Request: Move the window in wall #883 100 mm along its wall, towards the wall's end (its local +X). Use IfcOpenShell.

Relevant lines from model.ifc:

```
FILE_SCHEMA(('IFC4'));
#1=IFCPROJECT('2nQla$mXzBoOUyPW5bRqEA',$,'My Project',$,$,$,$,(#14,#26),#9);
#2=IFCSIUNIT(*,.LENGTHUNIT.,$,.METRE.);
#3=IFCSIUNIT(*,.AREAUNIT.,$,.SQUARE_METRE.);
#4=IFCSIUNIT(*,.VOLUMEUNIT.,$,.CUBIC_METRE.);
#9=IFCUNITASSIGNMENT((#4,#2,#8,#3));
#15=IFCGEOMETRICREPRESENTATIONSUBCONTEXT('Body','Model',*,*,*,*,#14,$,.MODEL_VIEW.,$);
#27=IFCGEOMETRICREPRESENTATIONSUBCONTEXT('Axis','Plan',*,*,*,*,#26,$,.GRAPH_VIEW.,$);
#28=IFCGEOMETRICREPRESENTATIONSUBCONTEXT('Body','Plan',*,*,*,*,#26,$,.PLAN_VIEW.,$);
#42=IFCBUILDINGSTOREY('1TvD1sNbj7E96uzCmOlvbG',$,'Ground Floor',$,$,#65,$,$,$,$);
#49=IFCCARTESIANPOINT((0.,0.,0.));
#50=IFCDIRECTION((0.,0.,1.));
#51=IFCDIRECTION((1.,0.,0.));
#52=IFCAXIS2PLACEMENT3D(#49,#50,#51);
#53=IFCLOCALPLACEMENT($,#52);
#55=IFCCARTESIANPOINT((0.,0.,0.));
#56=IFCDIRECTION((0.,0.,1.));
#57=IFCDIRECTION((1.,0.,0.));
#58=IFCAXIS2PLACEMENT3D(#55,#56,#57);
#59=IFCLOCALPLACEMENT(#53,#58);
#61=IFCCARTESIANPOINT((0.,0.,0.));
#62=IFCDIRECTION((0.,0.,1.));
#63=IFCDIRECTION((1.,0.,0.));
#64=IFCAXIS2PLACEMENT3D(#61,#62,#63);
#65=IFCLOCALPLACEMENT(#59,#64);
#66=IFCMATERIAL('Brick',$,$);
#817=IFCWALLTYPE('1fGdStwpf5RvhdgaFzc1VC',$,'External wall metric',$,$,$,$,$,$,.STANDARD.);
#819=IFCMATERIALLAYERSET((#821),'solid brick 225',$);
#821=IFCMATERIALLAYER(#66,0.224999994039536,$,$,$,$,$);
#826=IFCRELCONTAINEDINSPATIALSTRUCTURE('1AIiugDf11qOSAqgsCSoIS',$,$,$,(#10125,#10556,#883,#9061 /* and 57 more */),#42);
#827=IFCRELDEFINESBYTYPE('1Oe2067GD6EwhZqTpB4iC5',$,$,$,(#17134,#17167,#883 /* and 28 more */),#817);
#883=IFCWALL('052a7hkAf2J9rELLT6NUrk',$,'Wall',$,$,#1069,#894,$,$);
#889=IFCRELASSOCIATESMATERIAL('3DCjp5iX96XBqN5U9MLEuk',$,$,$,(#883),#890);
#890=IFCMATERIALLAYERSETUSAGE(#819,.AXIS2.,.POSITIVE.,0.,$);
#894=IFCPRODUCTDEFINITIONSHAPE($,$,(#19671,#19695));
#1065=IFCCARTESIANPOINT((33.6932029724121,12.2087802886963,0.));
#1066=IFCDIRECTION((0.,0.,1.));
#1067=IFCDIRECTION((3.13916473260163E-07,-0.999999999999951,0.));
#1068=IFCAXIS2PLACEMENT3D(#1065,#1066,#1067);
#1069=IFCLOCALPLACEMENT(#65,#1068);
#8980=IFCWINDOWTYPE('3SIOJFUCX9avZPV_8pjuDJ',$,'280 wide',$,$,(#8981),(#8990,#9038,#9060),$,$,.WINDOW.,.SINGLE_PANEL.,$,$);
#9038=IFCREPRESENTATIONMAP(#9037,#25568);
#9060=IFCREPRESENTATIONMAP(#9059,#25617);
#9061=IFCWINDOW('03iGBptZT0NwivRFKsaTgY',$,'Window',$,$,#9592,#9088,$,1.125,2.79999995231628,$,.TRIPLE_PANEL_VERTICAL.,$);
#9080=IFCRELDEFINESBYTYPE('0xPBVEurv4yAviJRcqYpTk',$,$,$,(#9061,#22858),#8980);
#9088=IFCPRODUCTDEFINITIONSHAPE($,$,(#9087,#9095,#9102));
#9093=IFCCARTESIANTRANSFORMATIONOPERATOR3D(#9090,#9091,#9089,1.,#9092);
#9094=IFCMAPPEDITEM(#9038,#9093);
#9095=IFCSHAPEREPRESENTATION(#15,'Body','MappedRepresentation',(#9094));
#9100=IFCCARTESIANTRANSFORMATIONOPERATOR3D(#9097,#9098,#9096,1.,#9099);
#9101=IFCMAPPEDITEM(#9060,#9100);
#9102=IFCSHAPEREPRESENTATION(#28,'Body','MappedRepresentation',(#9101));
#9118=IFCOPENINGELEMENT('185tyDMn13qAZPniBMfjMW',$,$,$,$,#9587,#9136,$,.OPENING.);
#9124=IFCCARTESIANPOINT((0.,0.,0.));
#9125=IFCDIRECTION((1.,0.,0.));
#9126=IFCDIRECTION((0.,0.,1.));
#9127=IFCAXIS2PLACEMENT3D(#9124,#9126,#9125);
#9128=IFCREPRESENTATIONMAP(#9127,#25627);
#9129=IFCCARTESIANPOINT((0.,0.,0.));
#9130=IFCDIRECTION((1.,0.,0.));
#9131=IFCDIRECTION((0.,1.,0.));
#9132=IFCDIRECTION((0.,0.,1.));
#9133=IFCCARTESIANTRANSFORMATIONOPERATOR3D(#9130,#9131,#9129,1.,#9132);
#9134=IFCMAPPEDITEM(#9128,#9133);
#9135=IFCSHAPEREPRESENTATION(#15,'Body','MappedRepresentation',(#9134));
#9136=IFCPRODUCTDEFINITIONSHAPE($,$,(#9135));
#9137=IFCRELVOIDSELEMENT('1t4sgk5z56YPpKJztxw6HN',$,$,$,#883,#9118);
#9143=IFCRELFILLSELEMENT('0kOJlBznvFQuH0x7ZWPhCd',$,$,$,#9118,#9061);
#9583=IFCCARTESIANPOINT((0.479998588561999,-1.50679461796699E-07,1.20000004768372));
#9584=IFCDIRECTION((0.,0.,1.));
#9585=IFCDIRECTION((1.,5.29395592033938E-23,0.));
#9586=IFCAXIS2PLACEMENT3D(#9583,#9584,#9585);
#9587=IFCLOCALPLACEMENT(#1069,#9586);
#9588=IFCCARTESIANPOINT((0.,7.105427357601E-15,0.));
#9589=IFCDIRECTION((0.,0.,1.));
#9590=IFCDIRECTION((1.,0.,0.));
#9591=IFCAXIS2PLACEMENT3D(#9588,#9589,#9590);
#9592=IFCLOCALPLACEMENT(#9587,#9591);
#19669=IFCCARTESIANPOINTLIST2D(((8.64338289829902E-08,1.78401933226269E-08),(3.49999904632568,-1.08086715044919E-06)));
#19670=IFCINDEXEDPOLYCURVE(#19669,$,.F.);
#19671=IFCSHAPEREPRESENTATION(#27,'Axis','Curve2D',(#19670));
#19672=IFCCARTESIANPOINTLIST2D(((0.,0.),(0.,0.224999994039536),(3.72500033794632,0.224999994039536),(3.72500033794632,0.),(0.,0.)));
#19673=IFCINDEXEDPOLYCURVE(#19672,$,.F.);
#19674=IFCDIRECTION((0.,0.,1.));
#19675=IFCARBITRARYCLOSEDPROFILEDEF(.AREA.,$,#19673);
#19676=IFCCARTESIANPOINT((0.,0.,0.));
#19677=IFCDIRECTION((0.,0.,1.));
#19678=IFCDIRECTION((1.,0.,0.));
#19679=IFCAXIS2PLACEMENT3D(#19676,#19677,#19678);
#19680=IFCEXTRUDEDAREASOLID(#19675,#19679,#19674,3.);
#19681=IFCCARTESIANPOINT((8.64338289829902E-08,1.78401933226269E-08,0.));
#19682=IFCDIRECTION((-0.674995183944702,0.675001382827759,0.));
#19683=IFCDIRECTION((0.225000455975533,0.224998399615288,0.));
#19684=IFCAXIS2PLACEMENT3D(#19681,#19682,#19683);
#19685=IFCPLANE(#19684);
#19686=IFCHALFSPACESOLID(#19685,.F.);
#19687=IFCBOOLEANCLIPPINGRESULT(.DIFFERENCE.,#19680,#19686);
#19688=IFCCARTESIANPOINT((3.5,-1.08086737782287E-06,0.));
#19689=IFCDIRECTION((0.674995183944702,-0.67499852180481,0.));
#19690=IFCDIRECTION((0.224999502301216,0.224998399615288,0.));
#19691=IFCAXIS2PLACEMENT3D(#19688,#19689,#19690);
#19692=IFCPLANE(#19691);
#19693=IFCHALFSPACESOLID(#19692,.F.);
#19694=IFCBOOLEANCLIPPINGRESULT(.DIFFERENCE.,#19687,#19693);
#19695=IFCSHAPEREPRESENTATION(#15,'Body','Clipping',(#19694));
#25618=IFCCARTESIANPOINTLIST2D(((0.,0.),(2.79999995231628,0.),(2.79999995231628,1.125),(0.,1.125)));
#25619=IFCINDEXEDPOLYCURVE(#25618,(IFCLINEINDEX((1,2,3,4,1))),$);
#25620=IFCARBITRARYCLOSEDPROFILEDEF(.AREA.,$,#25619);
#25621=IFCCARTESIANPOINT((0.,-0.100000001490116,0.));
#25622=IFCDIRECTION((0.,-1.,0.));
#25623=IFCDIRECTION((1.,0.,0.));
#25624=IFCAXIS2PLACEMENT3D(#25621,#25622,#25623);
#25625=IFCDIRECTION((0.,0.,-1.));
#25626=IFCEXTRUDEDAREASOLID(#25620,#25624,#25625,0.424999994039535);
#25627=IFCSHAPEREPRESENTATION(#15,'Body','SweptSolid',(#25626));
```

```python
import ifcopenshell
import ifcopenshell.api.geometry
import ifcopenshell.util.placement
import ifcopenshell.util.unit

model = ifcopenshell.open("model.ifc")
unit_scale = ifcopenshell.util.unit.calculate_unit_scale(model)

window = model.by_guid("03iGBptZT0NwivRFKsaTgY")
opening = window.FillsVoids[0].RelatingOpeningElement
wall = opening.VoidsElements[0].RelatingBuildingElement

wall_matrix = ifcopenshell.util.placement.get_local_placement(wall.ObjectPlacement)
shift = wall_matrix[:3, 0] * 0.1 / unit_scale
before = ifcopenshell.util.placement.get_local_placement(window.ObjectPlacement)[:3, 3].copy()

# The window is placed relative to its opening, so it follows when the opening moves.
matrix = ifcopenshell.util.placement.get_local_placement(opening.ObjectPlacement)
matrix[:3, 3] += shift
ifcopenshell.api.geometry.edit_object_placement(
    model, product=opening, matrix=matrix, is_si=False, should_transform_children=True
)

after = ifcopenshell.util.placement.get_local_placement(window.ObjectPlacement)[:3, 3]
print("window moved by", (after - before).round(3) + 0.0)

model.write("model_updated.ifc")
```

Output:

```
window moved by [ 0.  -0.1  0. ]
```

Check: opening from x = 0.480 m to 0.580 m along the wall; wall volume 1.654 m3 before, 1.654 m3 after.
